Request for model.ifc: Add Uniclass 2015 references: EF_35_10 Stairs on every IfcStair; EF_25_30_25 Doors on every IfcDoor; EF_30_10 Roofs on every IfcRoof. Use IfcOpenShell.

First a look at what the model holds.

```python
import ifcopenshell

model = ifcopenshell.open("model.ifc")
print(model.schema)
print("classifications:", [c.Name for c in model.by_type("IfcClassification")])
for ifc_class in ("IfcDoor", "IfcRoof", "IfcStair", "IfcWall", "IfcWindow"):
    print(ifc_class, len(model.by_type(ifc_class)))
```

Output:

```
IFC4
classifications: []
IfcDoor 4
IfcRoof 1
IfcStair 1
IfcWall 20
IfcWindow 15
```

```python
import ifcopenshell
import ifcopenshell.api.classification

model = ifcopenshell.open("model.ifc")

system = ifcopenshell.api.classification.add_classification(model, classification="Uniclass 2015")

codes = {
    "IfcStair": ("EF_35_10", "Stairs"),
    "IfcDoor": ("EF_25_30_25", "Doors"),
    "IfcRoof": ("EF_30_10", "Roofs"),
}
for ifc_class, (code, name) in codes.items():
    products = model.by_type(ifc_class)
    ifcopenshell.api.classification.add_reference(
        model, products=products, classification=system, identification=code, name=name
    )
    print(code, len(products))

model.write("model-out.ifc")
```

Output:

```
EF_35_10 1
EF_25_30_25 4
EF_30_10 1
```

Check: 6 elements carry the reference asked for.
